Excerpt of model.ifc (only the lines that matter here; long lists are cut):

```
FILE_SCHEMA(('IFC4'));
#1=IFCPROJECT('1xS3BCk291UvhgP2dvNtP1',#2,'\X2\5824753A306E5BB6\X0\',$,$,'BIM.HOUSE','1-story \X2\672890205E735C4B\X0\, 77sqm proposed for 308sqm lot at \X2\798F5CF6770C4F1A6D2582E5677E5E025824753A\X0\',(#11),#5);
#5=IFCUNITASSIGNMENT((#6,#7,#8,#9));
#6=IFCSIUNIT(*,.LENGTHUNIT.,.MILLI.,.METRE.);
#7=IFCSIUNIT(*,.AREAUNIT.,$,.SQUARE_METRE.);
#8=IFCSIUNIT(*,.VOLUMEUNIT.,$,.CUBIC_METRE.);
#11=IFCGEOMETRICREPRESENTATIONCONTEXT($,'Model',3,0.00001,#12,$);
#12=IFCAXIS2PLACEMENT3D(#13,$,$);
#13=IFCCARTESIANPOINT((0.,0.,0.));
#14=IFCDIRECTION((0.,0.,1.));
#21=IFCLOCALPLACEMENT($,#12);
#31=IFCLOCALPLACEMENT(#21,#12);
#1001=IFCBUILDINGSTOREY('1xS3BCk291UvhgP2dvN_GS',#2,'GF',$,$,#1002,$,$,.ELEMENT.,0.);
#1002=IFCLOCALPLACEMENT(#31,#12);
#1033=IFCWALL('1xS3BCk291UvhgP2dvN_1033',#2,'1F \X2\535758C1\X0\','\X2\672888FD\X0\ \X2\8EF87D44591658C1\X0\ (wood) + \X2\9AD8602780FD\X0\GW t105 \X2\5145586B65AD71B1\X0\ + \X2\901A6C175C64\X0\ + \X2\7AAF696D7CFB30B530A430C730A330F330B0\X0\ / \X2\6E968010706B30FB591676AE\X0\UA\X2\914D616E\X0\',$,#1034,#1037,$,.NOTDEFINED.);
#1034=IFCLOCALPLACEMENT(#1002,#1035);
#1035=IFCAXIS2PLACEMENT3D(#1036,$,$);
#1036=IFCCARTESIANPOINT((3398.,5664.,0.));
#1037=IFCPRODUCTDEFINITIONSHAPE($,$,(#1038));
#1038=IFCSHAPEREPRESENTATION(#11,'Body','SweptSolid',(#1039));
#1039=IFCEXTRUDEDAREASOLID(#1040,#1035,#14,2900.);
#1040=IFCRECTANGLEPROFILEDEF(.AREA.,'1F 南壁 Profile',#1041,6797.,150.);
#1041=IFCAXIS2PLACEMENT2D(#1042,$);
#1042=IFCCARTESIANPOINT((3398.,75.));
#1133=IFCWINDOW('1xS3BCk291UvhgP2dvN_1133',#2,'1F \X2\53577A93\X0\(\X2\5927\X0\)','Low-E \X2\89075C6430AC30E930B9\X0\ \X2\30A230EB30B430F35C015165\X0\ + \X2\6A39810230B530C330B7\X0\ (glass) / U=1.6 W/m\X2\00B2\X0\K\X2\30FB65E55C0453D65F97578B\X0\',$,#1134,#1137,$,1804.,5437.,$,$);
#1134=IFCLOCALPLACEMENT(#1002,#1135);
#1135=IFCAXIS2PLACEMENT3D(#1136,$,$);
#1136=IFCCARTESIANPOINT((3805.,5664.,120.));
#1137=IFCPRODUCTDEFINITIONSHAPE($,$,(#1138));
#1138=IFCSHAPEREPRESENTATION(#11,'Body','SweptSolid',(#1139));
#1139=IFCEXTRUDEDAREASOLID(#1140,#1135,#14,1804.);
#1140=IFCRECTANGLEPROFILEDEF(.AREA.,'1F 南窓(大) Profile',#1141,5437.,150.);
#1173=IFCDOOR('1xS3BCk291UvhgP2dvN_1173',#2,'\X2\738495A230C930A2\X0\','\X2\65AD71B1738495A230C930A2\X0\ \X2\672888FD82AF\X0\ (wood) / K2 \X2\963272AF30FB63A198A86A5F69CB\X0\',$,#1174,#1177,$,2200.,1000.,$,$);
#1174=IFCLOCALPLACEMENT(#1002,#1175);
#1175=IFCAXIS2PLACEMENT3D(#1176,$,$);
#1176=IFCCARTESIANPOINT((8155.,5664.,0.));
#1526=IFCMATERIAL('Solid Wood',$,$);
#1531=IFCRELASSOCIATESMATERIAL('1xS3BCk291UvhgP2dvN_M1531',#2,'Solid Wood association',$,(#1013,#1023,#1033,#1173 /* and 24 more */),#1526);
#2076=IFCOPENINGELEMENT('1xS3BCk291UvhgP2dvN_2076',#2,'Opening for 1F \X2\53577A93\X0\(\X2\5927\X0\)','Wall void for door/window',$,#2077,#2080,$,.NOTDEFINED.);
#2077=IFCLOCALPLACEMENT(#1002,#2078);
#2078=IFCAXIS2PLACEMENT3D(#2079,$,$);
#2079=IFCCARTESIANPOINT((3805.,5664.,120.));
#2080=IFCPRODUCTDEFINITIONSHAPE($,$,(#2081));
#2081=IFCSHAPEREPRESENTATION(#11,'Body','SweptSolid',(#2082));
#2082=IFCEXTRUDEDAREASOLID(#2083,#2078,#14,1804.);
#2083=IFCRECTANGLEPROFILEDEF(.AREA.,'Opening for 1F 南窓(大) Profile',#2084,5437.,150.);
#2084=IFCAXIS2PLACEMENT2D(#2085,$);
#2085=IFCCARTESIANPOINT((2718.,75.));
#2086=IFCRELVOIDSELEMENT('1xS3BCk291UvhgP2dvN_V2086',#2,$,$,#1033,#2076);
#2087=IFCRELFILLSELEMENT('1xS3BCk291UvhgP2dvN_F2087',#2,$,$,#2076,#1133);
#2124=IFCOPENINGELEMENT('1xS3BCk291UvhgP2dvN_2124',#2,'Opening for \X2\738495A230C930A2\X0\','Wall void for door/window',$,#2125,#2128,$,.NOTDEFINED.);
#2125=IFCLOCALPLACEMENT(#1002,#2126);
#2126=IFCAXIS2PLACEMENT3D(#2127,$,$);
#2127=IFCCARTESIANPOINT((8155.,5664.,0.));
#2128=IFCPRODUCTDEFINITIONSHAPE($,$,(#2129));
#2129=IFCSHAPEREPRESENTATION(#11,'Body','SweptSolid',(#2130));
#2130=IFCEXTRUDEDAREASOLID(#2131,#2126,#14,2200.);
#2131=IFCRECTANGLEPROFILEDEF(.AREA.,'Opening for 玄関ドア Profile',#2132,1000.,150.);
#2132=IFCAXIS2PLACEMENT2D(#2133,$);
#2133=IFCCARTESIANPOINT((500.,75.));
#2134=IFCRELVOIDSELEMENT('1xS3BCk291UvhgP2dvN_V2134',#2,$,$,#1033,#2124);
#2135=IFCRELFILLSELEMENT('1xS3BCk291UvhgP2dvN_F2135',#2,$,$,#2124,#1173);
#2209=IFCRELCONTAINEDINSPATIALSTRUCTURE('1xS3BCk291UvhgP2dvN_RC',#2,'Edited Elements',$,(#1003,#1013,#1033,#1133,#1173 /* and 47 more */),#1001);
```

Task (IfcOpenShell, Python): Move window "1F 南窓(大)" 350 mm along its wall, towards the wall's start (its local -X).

```python
import ifcopenshell
import ifcopenshell.api.geometry
import ifcopenshell.util.placement
import ifcopenshell.util.unit

model = ifcopenshell.open("model.ifc")
unit_scale = ifcopenshell.util.unit.calculate_unit_scale(model)

window = model.by_guid("1xS3BCk291UvhgP2dvN_1133")
opening = window.FillsVoids[0].RelatingOpeningElement
wall = opening.VoidsElements[0].RelatingBuildingElement

wall_matrix = ifcopenshell.util.placement.get_local_placement(wall.ObjectPlacement)
shift = wall_matrix[:3, 0] * -0.35 / unit_scale
before = ifcopenshell.util.placement.get_local_placement(window.ObjectPlacement)[:3, 3].copy()

# The window is not placed relative to its opening, so move both.
for product in (opening, window):
    matrix = ifcopenshell.util.placement.get_local_placement(product.ObjectPlacement)
    matrix[:3, 3] += shift
    ifcopenshell.api.geometry.edit_object_placement(model, product=product, matrix=matrix, is_si=False)

after = ifcopenshell.util.placement.get_local_placement(window.ObjectPlacement)[:3, 3]
print("window moved by", (after - before).round(3) + 0.0)

model.write("model-out.ifc")
```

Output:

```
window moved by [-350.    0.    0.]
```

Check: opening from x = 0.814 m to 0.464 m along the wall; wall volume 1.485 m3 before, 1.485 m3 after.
